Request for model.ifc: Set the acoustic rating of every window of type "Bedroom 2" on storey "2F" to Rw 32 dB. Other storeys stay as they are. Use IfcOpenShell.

First a look at what the model holds.

```python
import ifcopenshell
import ifcopenshell.util.element

model = ifcopenshell.open("model.ifc")
print(model.schema)
storey = next(s for s in model.by_type("IfcBuildingStorey") if s.Name == "2F")
windows = [e for e in ifcopenshell.util.element.get_decomposition(storey) if e.is_a("IfcWindow")]
seen = {}
for e in windows:
    element_type = ifcopenshell.util.element.get_type(e)
    key = (element_type.Name if element_type != e and element_type else None, ifcopenshell.util.element.get_pset(e, "Pset_WindowCommon", "AcousticRating"))
    seen[key] = seen.get(key, 0) + 1
for (name, value), count in sorted(seen.items(), key=str):
    print(count, "x", name, "|", value)
```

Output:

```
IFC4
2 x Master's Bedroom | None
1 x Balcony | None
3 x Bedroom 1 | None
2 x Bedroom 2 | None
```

```python
import ifcopenshell
import ifcopenshell.api.pset
import ifcopenshell.util.element

model = ifcopenshell.open("model.ifc")

storey = next(s for s in model.by_type("IfcBuildingStorey") if s.Name == "2F")
windows = [e for e in ifcopenshell.util.element.get_decomposition(storey) if e.is_a("IfcWindow")]

count = 0
for e in windows:
    element_type = ifcopenshell.util.element.get_type(e)
    if element_type in (None, e) or element_type.Name != "Bedroom 2":
        continue
    # add_pset returns the element's existing set when there is one.
    pset = ifcopenshell.api.pset.add_pset(model, product=e, name="Pset_WindowCommon")
    ifcopenshell.api.pset.edit_pset(model, pset=pset, properties={"AcousticRating": "Rw 32 dB"})
    count += 1

print(count, "windows updated")

model.write("model_v2.ifc")
```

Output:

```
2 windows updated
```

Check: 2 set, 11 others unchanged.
